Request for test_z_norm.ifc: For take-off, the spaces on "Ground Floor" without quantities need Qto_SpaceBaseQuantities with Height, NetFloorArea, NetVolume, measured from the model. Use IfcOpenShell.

First a look at what the model holds.

```python
import ifcopenshell
import ifcopenshell.util.element
import ifcopenshell.util.unit

model = ifcopenshell.open("test_z_norm.ifc")
print(model.schema)
for unit_type in ("LENGTHUNIT", "AREAUNIT", "VOLUMEUNIT"):
    print(unit_type, ifcopenshell.util.unit.calculate_unit_scale(model, unit_type))
storey = next(s for s in model.by_type("IfcBuildingStorey") if s.Name == "Ground Floor")
spaces = [e for e in ifcopenshell.util.element.get_decomposition(storey) if e.is_a("IfcSpace")]
for e in sorted(spaces, key=lambda e: e.id()):
    print(e.id(), e.is_a(), e.Name, list(ifcopenshell.util.element.get_psets(e, qtos_only=True)), sep=" | ")
```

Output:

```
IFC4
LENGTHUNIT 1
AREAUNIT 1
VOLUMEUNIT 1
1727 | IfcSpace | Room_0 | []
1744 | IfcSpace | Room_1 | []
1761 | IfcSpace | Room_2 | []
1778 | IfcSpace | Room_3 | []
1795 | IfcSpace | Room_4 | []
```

```python
import ifcopenshell
import ifcopenshell.api.pset
import ifcopenshell.geom
import ifcopenshell.util.element
import ifcopenshell.util.shape
import ifcopenshell.util.unit

model = ifcopenshell.open("test_z_norm.ifc")
unit_scale = ifcopenshell.util.unit.calculate_unit_scale(model)
area_scale = ifcopenshell.util.unit.calculate_unit_scale(model, "AREAUNIT")
volume_scale = ifcopenshell.util.unit.calculate_unit_scale(model, "VOLUMEUNIT")
settings = ifcopenshell.geom.settings()

storey = next(s for s in model.by_type("IfcBuildingStorey") if s.Name == "Ground Floor")
spaces = [e for e in ifcopenshell.util.element.get_decomposition(storey) if e.is_a("IfcSpace")]

for e in sorted(spaces, key=lambda e: e.id()):
    if ifcopenshell.util.element.get_psets(e, qtos_only=True, should_inherit=False):
        continue
    # Geometry comes back in metres, in the element's own axes.
    shape = ifcopenshell.geom.create_shape(settings, e)
    values = {
        "Height": ifcopenshell.util.shape.get_z(shape.geometry) / unit_scale,
        "NetFloorArea": ifcopenshell.util.shape.get_footprint_area(shape.geometry) / area_scale,
        "NetVolume": ifcopenshell.util.shape.get_volume(shape.geometry) / volume_scale,
    }
    qto = ifcopenshell.api.pset.add_qto(model, product=e, name="Qto_SpaceBaseQuantities")
    ifcopenshell.api.pset.edit_qto(model, qto=qto, properties=values)
    print(e.id(), {k: round(v, 3) for k, v in values.items()})

model.write("test_z_norm_updated.ifc")
```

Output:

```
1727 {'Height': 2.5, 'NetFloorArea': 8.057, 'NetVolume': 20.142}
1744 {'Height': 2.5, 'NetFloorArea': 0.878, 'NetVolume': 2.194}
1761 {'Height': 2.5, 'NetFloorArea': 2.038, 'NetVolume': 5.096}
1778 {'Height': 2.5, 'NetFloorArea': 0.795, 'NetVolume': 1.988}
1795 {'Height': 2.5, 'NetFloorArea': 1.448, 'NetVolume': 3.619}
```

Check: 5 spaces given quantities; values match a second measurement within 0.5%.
